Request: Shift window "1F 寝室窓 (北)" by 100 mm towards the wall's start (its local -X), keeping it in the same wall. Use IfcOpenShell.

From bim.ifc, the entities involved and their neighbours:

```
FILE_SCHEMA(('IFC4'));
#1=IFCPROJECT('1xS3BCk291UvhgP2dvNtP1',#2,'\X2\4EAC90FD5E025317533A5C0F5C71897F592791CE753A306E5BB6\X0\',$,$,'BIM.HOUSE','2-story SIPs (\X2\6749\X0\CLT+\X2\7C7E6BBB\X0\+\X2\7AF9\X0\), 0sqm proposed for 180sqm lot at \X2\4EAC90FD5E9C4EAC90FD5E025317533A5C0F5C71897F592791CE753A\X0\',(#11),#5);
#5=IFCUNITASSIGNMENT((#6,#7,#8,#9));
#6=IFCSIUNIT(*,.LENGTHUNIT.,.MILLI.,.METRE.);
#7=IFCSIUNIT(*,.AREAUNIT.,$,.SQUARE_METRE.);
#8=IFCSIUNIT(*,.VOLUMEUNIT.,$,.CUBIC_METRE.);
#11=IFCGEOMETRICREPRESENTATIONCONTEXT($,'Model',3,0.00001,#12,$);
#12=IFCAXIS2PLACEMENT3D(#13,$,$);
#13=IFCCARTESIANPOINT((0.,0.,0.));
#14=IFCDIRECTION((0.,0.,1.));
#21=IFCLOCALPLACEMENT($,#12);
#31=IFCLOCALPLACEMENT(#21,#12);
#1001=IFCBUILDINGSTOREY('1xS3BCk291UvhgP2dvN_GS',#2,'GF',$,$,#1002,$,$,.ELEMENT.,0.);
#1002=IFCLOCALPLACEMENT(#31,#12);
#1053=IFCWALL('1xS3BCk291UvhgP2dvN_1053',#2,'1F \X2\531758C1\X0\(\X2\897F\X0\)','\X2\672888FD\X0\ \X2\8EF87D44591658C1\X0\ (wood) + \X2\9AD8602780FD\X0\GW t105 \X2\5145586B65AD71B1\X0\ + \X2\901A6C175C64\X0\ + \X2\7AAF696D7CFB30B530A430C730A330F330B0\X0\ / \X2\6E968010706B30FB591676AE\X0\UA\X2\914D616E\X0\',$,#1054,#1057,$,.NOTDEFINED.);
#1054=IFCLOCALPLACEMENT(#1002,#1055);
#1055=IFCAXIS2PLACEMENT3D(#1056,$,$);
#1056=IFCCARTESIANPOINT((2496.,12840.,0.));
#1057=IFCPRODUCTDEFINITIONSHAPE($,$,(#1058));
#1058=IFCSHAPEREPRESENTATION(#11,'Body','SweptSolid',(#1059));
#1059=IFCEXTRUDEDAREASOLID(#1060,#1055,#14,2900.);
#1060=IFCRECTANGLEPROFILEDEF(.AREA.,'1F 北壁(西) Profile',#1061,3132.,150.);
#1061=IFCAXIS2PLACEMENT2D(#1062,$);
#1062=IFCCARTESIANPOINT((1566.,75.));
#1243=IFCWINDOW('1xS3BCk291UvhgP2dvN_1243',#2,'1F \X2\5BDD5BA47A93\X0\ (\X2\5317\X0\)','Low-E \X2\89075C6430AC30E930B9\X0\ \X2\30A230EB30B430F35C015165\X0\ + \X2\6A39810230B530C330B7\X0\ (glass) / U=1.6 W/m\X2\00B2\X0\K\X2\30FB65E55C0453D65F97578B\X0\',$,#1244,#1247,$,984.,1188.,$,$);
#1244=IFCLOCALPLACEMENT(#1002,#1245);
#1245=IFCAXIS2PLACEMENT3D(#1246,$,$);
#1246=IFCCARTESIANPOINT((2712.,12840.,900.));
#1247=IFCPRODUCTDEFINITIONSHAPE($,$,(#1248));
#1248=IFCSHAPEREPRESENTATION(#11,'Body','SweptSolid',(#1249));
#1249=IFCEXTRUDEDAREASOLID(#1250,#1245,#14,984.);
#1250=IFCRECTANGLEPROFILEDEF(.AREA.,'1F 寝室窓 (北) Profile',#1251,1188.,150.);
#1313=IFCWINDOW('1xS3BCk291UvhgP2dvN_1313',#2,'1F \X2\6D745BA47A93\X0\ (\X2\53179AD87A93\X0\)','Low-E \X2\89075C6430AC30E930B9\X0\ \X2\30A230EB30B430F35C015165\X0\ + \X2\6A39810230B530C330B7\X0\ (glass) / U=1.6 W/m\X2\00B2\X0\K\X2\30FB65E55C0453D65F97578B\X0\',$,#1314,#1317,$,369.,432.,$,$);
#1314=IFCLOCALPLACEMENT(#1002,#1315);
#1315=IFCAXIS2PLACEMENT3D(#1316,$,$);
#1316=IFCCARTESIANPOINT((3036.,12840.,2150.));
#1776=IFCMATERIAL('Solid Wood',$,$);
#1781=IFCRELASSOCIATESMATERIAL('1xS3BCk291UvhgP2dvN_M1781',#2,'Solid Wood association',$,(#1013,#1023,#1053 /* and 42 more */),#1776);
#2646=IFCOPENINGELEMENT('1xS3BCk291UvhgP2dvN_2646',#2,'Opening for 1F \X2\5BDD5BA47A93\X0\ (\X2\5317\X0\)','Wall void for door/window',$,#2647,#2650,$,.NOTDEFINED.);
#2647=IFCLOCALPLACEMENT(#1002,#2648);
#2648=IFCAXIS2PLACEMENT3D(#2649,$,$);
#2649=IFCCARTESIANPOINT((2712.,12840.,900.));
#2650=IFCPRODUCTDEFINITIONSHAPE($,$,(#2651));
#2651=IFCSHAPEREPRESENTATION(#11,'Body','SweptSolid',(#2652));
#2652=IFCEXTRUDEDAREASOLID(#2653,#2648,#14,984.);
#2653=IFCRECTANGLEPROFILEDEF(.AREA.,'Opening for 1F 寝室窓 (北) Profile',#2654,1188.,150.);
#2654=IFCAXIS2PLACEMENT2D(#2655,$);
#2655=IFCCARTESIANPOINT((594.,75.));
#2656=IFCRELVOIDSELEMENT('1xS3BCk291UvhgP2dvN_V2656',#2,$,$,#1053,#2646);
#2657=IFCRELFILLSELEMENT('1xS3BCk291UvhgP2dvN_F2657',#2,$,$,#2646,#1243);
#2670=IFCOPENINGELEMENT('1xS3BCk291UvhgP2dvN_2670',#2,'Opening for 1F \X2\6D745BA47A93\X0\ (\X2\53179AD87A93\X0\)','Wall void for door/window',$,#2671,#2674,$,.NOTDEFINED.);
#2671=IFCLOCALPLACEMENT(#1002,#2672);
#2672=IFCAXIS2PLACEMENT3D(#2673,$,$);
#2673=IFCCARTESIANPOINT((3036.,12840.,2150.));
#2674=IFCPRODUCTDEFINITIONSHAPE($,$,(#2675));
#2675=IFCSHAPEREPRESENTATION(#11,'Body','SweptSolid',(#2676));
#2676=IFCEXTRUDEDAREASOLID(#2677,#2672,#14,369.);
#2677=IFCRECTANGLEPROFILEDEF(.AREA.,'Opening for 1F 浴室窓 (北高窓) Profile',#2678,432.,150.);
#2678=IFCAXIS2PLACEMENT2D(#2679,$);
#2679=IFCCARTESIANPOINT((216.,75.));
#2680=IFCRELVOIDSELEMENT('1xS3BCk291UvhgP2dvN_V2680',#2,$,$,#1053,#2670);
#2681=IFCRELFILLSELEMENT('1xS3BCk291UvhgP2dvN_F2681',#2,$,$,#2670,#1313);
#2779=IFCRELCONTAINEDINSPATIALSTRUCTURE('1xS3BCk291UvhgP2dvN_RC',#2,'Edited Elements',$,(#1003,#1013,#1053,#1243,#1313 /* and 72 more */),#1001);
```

```python
import ifcopenshell
import ifcopenshell.api.geometry
import ifcopenshell.util.placement
import ifcopenshell.util.unit

model = ifcopenshell.open("bim.ifc")
unit_scale = ifcopenshell.util.unit.calculate_unit_scale(model)

window = model.by_id(1243)
opening = window.FillsVoids[0].RelatingOpeningElement
wall = opening.VoidsElements[0].RelatingBuildingElement

wall_matrix = ifcopenshell.util.placement.get_local_placement(wall.ObjectPlacement)
shift = wall_matrix[:3, 0] * -0.1 / unit_scale
before = ifcopenshell.util.placement.get_local_placement(window.ObjectPlacement)[:3, 3].copy()

# The window is not placed relative to its opening, so move both.
for product in (opening, window):
    matrix = ifcopenshell.util.placement.get_local_placement(product.ObjectPlacement)
    matrix[:3, 3] += shift
    ifcopenshell.api.geometry.edit_object_placement(model, product=product, matrix=matrix, is_si=False)

after = ifcopenshell.util.placement.get_local_placement(window.ObjectPlacement)[:3, 3]
print("window moved by", (after - before).round(3) + 0.0)

model.write("bim_updated.ifc")
```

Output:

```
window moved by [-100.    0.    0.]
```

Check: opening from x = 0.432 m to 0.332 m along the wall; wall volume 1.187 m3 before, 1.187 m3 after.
